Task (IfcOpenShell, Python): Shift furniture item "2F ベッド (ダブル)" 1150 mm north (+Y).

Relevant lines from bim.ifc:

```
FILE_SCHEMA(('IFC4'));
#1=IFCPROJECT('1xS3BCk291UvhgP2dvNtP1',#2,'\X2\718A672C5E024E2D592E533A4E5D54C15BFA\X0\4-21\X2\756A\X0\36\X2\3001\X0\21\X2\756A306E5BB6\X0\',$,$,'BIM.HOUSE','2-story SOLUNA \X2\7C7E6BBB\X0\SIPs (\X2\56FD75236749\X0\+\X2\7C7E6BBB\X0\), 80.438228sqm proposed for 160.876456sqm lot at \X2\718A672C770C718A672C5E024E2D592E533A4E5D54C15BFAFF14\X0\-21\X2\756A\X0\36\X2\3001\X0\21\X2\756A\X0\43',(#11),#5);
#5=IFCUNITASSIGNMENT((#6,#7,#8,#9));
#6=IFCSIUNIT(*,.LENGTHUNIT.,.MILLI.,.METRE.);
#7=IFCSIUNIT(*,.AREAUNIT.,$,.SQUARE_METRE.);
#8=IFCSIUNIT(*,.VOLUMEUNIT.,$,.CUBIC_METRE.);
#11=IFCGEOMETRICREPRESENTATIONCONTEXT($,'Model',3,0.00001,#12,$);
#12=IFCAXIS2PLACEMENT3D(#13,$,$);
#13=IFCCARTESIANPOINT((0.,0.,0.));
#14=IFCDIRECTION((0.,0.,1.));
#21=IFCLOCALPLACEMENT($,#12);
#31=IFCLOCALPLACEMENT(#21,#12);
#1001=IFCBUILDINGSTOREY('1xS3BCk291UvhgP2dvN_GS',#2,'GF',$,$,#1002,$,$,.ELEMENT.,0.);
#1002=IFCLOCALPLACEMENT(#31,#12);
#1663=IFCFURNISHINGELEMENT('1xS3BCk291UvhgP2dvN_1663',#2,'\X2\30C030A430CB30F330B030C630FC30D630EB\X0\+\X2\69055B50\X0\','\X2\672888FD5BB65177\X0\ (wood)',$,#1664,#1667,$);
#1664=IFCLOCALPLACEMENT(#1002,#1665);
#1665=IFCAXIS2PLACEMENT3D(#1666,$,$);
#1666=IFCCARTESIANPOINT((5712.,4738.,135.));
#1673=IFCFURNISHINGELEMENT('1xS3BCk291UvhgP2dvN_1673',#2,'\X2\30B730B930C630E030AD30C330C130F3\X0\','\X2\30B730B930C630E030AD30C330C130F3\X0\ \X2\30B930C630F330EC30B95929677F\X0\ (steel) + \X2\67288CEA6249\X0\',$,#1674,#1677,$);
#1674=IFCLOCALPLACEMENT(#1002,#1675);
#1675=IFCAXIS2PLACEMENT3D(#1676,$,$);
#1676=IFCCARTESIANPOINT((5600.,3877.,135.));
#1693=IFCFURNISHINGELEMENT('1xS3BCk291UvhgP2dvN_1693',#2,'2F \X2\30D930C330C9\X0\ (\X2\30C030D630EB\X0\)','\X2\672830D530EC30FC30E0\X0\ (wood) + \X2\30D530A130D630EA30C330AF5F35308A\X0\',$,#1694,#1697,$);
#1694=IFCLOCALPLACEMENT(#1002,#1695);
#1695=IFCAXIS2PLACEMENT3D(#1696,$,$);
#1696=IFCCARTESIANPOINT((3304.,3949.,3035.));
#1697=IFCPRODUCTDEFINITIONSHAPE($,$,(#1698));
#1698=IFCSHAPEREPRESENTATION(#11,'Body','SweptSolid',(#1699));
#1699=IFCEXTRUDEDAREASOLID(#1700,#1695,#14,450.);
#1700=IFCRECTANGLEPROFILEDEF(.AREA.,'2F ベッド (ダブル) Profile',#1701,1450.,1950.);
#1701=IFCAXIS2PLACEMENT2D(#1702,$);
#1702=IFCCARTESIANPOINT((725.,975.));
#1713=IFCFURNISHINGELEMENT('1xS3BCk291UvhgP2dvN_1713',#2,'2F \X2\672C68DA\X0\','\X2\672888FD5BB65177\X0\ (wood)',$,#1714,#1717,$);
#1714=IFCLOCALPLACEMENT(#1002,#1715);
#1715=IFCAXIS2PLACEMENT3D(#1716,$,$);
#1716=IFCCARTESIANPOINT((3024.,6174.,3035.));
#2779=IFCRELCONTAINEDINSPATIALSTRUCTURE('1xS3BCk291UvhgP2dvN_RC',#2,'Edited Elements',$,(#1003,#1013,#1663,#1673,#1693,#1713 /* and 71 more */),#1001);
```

```python
import ifcopenshell
import ifcopenshell.api.geometry
import ifcopenshell.util.placement
import ifcopenshell.util.unit

model = ifcopenshell.open("bim.ifc")
unit_scale = ifcopenshell.util.unit.calculate_unit_scale(model)

item = model.by_guid("1xS3BCk291UvhgP2dvN_1693")
matrix = ifcopenshell.util.placement.get_local_placement(item.ObjectPlacement)
matrix[1, 3] += 1.15 / unit_scale
ifcopenshell.api.geometry.edit_object_placement(model, product=item, matrix=matrix, is_si=False)

print(ifcopenshell.util.placement.get_local_placement(item.ObjectPlacement).round(3) + 0.0)

model.write("bim_rev.ifc")
```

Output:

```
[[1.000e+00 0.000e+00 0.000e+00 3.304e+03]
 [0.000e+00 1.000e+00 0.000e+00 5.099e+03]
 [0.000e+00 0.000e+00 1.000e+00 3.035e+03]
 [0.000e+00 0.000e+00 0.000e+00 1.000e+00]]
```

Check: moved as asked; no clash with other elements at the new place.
